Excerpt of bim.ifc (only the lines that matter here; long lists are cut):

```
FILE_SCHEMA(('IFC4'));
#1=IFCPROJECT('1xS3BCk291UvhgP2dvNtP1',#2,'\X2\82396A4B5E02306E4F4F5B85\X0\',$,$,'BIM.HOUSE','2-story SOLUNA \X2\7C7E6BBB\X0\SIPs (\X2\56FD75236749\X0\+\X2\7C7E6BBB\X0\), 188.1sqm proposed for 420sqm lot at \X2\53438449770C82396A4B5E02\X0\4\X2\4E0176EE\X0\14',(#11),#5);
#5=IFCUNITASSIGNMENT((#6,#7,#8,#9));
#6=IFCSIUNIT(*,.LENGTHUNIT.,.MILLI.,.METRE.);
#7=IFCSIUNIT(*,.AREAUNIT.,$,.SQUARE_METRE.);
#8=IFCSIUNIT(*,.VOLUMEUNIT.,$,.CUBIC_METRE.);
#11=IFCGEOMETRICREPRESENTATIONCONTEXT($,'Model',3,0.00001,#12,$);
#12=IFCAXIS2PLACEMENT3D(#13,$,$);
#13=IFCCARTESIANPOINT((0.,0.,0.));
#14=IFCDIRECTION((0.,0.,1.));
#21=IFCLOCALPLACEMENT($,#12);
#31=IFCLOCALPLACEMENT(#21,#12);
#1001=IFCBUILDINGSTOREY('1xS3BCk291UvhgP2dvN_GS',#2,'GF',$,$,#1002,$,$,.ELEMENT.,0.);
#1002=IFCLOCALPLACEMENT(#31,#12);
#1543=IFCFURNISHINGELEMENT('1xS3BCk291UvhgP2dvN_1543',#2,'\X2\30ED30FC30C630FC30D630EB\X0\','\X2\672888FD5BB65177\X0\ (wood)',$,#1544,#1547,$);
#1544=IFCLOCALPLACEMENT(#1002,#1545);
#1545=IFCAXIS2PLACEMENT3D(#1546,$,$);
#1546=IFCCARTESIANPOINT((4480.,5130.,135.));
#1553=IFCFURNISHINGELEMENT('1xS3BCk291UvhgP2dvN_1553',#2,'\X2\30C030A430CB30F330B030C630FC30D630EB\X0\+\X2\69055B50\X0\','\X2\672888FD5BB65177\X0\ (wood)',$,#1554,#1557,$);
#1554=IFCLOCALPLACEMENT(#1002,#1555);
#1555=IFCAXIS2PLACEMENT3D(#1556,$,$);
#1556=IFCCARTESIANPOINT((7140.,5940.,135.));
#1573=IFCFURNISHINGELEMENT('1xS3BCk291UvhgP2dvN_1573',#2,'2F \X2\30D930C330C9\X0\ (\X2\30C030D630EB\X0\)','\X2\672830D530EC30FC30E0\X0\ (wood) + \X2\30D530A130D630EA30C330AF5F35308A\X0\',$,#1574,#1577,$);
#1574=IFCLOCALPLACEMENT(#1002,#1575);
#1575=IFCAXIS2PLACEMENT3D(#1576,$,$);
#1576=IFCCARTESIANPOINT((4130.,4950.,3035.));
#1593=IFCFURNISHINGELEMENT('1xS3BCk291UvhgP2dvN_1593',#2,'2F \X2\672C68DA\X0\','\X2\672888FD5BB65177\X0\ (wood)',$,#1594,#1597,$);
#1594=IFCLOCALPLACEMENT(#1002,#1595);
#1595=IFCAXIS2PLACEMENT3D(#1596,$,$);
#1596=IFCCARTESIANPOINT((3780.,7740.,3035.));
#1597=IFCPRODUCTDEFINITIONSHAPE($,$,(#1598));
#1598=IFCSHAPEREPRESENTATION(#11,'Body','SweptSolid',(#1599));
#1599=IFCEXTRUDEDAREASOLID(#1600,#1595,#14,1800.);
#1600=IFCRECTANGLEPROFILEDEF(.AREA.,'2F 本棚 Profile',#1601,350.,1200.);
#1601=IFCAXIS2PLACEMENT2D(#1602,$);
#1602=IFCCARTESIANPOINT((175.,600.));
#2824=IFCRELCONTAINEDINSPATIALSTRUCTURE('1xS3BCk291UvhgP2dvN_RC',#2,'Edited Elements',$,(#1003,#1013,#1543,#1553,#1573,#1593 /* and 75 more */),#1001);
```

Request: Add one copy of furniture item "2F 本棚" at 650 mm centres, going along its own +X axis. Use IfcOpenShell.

```python
import ifcopenshell
import ifcopenshell.api.geometry
import ifcopenshell.api.root
import ifcopenshell.util.element
import ifcopenshell.util.placement
import ifcopenshell.util.unit

model = ifcopenshell.open("bim.ifc")
unit_scale = ifcopenshell.util.unit.calculate_unit_scale(model)


def reuse_history(source, copy):
    """copy_class also copies each property set's owner history, people and application; keep the originals."""
    for rel in copy.IsDefinedBy:
        if rel.is_a("IfcRelDefinesByProperties") and (history := rel.RelatingPropertyDefinition.OwnerHistory):
            rel.RelatingPropertyDefinition.OwnerHistory = source.OwnerHistory
            ifcopenshell.util.element.remove_deep2(model, history)


source = model.by_id(1593)
base = ifcopenshell.util.placement.get_local_placement(source.ObjectPlacement)
step = base[:3, 0] * 0.65 / unit_scale

for i in range(1, 2):
    copy = ifcopenshell.api.root.copy_class(model, product=source)
    copy.Representation = ifcopenshell.util.element.copy_deep(
        model, source.Representation, exclude=["IfcGeometricRepresentationContext", "IfcRepresentationMap"]
    )
    reuse_history(source, copy)
    matrix = base.copy()
    matrix[:3, 3] += i * step
    print("added at", matrix[:3, 3].round(3) + 0.0)
    ifcopenshell.api.geometry.edit_object_placement(model, product=copy, matrix=matrix, is_si=False)

model.write("bim_rev.ifc")
```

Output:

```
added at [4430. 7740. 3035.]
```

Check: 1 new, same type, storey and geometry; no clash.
